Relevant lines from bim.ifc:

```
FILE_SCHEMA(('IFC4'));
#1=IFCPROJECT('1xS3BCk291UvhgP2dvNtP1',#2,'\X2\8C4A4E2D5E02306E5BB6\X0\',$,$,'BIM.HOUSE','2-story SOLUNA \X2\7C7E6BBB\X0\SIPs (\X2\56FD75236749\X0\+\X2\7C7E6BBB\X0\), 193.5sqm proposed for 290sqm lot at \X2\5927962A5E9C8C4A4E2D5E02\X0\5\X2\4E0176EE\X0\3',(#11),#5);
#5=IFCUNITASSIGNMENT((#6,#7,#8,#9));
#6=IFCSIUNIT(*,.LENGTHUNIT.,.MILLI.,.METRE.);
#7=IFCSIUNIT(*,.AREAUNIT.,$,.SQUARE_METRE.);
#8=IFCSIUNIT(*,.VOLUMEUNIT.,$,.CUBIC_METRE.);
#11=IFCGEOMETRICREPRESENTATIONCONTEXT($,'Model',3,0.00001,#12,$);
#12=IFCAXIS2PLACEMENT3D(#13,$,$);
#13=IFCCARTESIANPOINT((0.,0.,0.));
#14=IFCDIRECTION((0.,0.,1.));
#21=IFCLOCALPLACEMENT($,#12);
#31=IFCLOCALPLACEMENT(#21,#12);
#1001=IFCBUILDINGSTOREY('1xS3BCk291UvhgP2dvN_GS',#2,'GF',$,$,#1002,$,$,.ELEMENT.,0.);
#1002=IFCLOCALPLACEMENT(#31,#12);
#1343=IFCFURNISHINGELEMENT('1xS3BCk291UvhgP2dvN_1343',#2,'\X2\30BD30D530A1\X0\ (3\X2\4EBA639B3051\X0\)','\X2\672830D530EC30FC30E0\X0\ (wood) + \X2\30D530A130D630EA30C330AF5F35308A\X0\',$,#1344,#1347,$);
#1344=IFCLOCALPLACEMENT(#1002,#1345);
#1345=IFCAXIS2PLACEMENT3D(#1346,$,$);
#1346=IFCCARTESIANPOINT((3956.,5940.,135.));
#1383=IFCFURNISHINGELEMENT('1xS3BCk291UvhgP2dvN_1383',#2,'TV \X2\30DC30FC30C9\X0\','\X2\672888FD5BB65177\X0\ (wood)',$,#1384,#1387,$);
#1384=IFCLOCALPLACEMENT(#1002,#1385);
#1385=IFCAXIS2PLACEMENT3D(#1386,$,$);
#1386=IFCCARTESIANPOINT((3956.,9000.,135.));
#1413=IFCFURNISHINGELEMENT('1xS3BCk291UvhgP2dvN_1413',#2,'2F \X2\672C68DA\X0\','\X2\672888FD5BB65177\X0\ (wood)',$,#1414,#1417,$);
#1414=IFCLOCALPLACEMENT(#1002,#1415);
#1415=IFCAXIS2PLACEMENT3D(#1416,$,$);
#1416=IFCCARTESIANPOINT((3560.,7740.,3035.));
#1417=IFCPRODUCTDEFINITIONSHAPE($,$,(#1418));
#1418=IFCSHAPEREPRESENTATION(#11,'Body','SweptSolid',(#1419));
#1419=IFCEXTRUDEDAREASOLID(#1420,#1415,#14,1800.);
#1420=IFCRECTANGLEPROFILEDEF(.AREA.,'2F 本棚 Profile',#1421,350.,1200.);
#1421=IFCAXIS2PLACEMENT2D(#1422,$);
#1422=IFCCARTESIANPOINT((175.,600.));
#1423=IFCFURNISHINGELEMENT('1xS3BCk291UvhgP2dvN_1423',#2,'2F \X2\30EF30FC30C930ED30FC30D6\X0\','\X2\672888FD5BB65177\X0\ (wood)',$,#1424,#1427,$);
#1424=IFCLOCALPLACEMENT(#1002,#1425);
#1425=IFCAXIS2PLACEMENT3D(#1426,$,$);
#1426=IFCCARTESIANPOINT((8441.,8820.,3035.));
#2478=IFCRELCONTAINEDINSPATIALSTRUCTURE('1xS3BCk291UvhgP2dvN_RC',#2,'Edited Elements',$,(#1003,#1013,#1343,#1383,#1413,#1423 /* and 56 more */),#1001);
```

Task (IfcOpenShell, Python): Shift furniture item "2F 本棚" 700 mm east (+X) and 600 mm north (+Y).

```python
import ifcopenshell
import ifcopenshell.api.geometry
import ifcopenshell.util.placement

model = ifcopenshell.open("bim.ifc")

item = model.by_guid("1xS3BCk291UvhgP2dvN_1413")
matrix = ifcopenshell.util.placement.get_local_placement(item.ObjectPlacement)
matrix[0, 3] += 700.0
matrix[1, 3] += 600.0
ifcopenshell.api.geometry.edit_object_placement(model, product=item, matrix=matrix, is_si=False)

print(ifcopenshell.util.placement.get_local_placement(item.ObjectPlacement).round(3) + 0.0)

model.write("bim_updated.ifc")
```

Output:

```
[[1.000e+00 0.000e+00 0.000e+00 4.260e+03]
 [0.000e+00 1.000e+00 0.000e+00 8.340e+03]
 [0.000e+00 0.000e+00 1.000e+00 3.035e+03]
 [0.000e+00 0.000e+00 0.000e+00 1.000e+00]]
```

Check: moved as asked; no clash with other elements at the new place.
